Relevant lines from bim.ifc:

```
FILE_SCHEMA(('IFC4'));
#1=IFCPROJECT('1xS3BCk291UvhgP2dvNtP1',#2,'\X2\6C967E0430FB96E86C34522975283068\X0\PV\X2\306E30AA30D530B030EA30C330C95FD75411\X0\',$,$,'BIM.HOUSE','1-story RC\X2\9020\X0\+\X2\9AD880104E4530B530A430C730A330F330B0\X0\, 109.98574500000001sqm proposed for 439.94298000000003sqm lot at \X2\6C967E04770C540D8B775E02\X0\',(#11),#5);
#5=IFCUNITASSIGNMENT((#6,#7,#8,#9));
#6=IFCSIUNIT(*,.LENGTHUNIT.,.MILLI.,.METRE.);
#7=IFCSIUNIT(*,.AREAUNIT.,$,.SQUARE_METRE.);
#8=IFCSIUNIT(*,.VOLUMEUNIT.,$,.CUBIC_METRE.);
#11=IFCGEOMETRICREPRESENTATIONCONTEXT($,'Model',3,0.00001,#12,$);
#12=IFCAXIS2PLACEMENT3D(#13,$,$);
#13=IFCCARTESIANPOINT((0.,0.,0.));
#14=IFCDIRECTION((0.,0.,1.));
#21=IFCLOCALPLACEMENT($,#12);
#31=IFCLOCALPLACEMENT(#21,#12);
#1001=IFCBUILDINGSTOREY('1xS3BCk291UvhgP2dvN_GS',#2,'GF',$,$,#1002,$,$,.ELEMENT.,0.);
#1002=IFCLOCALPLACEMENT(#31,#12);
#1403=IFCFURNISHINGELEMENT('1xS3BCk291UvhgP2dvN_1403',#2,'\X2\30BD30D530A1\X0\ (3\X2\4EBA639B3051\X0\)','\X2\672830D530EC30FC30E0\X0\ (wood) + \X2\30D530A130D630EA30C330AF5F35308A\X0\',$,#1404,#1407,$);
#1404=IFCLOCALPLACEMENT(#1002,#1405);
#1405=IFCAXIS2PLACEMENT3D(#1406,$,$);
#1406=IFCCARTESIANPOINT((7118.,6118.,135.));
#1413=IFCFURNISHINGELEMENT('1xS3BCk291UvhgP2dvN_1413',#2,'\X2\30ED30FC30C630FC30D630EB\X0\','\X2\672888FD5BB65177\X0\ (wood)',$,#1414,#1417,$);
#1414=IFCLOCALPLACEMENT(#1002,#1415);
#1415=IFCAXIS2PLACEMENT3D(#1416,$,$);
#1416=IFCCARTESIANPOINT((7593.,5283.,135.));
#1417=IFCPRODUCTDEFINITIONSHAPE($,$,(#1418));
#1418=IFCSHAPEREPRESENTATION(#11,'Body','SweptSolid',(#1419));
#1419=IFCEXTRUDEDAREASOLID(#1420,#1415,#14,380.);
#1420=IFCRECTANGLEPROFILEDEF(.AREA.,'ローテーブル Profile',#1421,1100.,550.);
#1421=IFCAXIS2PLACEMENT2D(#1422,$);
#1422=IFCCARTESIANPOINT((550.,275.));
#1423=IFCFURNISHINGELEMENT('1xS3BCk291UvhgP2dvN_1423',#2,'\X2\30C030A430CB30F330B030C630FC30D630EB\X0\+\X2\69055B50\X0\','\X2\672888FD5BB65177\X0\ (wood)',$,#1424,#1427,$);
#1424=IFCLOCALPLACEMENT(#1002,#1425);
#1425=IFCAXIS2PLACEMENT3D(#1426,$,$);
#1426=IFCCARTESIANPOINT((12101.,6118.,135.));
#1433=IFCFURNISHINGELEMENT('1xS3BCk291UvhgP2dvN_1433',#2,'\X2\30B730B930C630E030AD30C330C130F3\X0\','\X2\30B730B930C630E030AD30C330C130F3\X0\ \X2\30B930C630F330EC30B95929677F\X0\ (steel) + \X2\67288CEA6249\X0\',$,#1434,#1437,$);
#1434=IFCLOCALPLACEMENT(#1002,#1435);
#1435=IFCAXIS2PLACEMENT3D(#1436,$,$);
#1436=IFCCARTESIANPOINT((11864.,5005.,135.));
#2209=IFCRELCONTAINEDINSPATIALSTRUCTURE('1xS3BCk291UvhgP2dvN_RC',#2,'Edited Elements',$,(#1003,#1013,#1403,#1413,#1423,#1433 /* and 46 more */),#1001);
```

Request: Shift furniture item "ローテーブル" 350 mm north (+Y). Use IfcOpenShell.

```python
import ifcopenshell
import ifcopenshell.api.geometry
import ifcopenshell.util.placement
import ifcopenshell.util.unit

model = ifcopenshell.open("bim.ifc")
unit_scale = ifcopenshell.util.unit.calculate_unit_scale(model)

item = model.by_guid("1xS3BCk291UvhgP2dvN_1413")
matrix = ifcopenshell.util.placement.get_local_placement(item.ObjectPlacement)
matrix[1, 3] += 0.35 / unit_scale
ifcopenshell.api.geometry.edit_object_placement(model, product=item, matrix=matrix, is_si=False)

print(ifcopenshell.util.placement.get_local_placement(item.ObjectPlacement).round(3) + 0.0)

model.write("bim-out.ifc")
```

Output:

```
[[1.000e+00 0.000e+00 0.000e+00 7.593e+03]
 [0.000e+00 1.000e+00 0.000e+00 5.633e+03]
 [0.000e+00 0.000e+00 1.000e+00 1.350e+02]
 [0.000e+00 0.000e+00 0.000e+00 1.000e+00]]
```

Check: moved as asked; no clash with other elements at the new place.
